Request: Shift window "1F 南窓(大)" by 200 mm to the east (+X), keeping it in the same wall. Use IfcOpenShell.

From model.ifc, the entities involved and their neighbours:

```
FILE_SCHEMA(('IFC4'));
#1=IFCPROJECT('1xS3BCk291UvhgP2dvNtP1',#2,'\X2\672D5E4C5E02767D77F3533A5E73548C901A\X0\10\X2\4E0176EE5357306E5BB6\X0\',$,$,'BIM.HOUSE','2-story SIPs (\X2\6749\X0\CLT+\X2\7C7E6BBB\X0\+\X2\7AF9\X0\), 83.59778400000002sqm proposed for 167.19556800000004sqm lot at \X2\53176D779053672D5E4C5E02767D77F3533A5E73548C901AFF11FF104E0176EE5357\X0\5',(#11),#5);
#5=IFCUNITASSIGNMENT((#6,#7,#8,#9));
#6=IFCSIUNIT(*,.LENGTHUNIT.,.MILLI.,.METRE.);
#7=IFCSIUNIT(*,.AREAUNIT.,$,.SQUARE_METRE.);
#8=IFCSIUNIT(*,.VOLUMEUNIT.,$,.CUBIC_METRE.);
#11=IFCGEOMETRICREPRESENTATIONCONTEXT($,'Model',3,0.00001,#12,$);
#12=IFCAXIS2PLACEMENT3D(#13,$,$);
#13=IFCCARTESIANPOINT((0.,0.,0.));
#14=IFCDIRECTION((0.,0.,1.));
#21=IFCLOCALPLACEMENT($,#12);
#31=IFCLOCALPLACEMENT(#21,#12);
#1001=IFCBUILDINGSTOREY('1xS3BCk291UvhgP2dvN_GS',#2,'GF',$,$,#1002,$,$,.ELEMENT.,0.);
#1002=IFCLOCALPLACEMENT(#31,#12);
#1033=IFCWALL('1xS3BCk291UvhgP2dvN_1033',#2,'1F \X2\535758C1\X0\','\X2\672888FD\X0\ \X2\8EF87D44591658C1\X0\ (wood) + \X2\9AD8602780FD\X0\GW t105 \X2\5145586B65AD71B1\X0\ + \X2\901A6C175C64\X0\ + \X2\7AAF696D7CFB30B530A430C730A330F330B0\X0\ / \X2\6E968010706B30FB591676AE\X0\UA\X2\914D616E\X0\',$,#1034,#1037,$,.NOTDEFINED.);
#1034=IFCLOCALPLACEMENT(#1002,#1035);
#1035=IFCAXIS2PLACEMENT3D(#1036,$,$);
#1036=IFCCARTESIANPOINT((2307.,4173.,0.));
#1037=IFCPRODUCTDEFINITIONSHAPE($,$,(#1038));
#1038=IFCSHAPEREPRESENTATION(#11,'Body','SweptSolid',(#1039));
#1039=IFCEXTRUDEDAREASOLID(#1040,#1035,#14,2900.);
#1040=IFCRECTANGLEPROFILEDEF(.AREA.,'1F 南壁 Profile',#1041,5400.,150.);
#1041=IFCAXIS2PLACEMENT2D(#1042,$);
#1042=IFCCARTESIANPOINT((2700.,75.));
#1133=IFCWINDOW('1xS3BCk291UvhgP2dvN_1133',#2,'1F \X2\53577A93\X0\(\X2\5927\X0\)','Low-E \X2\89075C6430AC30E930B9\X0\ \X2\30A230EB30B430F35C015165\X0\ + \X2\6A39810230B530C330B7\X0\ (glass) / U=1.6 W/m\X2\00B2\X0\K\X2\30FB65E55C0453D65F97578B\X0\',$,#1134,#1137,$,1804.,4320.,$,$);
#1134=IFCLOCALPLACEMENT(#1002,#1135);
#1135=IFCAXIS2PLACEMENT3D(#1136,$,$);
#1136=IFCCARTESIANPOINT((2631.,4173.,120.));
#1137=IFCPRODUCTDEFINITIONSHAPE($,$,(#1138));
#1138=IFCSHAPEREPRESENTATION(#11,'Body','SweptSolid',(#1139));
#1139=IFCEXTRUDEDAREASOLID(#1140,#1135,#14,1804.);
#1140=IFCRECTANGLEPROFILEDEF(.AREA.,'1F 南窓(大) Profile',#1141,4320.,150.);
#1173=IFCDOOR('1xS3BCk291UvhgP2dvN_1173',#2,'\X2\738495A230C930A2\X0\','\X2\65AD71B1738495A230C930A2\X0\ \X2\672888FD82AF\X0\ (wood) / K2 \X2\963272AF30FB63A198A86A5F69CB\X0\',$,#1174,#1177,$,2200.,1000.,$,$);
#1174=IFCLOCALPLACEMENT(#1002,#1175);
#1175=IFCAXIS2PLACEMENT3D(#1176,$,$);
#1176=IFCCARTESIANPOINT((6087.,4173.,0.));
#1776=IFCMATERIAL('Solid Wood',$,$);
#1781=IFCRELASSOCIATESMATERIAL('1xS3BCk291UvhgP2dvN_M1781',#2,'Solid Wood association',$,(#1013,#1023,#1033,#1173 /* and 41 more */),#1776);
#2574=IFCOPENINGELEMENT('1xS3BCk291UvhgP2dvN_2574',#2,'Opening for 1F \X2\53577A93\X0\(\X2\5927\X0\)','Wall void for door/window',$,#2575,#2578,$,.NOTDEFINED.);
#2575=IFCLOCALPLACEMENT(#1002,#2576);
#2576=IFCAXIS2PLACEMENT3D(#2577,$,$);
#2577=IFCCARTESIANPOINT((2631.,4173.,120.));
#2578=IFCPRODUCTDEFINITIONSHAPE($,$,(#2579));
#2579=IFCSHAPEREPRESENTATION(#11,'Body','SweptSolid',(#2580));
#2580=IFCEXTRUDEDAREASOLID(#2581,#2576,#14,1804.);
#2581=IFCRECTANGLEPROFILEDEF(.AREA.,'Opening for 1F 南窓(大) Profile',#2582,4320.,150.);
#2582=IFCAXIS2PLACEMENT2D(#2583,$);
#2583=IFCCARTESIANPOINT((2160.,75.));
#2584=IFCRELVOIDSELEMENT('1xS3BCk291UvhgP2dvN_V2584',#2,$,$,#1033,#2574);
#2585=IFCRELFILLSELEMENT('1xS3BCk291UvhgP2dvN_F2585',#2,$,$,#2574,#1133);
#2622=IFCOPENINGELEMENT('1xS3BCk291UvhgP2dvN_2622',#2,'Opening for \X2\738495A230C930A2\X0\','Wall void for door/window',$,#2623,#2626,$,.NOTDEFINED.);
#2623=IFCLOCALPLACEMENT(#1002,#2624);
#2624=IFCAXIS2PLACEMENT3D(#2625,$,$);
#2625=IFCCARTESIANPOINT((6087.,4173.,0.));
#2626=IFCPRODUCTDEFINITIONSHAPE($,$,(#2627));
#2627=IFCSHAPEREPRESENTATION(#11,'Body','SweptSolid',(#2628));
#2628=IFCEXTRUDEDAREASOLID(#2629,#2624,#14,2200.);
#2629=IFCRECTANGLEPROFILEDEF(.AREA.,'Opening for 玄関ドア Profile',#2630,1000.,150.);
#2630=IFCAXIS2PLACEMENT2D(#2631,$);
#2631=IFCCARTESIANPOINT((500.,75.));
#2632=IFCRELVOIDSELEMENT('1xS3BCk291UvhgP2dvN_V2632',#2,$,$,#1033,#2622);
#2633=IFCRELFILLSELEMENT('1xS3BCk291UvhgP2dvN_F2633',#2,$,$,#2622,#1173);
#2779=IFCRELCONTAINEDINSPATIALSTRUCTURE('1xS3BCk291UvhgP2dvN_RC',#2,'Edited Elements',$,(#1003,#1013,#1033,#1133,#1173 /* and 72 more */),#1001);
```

```python
import ifcopenshell
import ifcopenshell.api.geometry
import ifcopenshell.util.placement
import ifcopenshell.util.unit

model = ifcopenshell.open("model.ifc")
unit_scale = ifcopenshell.util.unit.calculate_unit_scale(model)

window = model.by_guid("1xS3BCk291UvhgP2dvN_1133")
opening = window.FillsVoids[0].RelatingOpeningElement
wall = opening.VoidsElements[0].RelatingBuildingElement

wall_matrix = ifcopenshell.util.placement.get_local_placement(wall.ObjectPlacement)
shift = wall_matrix[:3, 0] * 0.2 / unit_scale
before = ifcopenshell.util.placement.get_local_placement(window.ObjectPlacement)[:3, 3].copy()

# The window is not placed relative to its opening, so move both.
for product in (opening, window):
    matrix = ifcopenshell.util.placement.get_local_placement(product.ObjectPlacement)
    matrix[:3, 3] += shift
    ifcopenshell.api.geometry.edit_object_placement(model, product=product, matrix=matrix, is_si=False)

after = ifcopenshell.util.placement.get_local_placement(window.ObjectPlacement)[:3, 3]
print("window moved by", (after - before).round(3) + 0.0)

model.write("model_rev.ifc")
```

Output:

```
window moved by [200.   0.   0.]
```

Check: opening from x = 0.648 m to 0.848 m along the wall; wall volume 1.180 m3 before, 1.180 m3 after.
